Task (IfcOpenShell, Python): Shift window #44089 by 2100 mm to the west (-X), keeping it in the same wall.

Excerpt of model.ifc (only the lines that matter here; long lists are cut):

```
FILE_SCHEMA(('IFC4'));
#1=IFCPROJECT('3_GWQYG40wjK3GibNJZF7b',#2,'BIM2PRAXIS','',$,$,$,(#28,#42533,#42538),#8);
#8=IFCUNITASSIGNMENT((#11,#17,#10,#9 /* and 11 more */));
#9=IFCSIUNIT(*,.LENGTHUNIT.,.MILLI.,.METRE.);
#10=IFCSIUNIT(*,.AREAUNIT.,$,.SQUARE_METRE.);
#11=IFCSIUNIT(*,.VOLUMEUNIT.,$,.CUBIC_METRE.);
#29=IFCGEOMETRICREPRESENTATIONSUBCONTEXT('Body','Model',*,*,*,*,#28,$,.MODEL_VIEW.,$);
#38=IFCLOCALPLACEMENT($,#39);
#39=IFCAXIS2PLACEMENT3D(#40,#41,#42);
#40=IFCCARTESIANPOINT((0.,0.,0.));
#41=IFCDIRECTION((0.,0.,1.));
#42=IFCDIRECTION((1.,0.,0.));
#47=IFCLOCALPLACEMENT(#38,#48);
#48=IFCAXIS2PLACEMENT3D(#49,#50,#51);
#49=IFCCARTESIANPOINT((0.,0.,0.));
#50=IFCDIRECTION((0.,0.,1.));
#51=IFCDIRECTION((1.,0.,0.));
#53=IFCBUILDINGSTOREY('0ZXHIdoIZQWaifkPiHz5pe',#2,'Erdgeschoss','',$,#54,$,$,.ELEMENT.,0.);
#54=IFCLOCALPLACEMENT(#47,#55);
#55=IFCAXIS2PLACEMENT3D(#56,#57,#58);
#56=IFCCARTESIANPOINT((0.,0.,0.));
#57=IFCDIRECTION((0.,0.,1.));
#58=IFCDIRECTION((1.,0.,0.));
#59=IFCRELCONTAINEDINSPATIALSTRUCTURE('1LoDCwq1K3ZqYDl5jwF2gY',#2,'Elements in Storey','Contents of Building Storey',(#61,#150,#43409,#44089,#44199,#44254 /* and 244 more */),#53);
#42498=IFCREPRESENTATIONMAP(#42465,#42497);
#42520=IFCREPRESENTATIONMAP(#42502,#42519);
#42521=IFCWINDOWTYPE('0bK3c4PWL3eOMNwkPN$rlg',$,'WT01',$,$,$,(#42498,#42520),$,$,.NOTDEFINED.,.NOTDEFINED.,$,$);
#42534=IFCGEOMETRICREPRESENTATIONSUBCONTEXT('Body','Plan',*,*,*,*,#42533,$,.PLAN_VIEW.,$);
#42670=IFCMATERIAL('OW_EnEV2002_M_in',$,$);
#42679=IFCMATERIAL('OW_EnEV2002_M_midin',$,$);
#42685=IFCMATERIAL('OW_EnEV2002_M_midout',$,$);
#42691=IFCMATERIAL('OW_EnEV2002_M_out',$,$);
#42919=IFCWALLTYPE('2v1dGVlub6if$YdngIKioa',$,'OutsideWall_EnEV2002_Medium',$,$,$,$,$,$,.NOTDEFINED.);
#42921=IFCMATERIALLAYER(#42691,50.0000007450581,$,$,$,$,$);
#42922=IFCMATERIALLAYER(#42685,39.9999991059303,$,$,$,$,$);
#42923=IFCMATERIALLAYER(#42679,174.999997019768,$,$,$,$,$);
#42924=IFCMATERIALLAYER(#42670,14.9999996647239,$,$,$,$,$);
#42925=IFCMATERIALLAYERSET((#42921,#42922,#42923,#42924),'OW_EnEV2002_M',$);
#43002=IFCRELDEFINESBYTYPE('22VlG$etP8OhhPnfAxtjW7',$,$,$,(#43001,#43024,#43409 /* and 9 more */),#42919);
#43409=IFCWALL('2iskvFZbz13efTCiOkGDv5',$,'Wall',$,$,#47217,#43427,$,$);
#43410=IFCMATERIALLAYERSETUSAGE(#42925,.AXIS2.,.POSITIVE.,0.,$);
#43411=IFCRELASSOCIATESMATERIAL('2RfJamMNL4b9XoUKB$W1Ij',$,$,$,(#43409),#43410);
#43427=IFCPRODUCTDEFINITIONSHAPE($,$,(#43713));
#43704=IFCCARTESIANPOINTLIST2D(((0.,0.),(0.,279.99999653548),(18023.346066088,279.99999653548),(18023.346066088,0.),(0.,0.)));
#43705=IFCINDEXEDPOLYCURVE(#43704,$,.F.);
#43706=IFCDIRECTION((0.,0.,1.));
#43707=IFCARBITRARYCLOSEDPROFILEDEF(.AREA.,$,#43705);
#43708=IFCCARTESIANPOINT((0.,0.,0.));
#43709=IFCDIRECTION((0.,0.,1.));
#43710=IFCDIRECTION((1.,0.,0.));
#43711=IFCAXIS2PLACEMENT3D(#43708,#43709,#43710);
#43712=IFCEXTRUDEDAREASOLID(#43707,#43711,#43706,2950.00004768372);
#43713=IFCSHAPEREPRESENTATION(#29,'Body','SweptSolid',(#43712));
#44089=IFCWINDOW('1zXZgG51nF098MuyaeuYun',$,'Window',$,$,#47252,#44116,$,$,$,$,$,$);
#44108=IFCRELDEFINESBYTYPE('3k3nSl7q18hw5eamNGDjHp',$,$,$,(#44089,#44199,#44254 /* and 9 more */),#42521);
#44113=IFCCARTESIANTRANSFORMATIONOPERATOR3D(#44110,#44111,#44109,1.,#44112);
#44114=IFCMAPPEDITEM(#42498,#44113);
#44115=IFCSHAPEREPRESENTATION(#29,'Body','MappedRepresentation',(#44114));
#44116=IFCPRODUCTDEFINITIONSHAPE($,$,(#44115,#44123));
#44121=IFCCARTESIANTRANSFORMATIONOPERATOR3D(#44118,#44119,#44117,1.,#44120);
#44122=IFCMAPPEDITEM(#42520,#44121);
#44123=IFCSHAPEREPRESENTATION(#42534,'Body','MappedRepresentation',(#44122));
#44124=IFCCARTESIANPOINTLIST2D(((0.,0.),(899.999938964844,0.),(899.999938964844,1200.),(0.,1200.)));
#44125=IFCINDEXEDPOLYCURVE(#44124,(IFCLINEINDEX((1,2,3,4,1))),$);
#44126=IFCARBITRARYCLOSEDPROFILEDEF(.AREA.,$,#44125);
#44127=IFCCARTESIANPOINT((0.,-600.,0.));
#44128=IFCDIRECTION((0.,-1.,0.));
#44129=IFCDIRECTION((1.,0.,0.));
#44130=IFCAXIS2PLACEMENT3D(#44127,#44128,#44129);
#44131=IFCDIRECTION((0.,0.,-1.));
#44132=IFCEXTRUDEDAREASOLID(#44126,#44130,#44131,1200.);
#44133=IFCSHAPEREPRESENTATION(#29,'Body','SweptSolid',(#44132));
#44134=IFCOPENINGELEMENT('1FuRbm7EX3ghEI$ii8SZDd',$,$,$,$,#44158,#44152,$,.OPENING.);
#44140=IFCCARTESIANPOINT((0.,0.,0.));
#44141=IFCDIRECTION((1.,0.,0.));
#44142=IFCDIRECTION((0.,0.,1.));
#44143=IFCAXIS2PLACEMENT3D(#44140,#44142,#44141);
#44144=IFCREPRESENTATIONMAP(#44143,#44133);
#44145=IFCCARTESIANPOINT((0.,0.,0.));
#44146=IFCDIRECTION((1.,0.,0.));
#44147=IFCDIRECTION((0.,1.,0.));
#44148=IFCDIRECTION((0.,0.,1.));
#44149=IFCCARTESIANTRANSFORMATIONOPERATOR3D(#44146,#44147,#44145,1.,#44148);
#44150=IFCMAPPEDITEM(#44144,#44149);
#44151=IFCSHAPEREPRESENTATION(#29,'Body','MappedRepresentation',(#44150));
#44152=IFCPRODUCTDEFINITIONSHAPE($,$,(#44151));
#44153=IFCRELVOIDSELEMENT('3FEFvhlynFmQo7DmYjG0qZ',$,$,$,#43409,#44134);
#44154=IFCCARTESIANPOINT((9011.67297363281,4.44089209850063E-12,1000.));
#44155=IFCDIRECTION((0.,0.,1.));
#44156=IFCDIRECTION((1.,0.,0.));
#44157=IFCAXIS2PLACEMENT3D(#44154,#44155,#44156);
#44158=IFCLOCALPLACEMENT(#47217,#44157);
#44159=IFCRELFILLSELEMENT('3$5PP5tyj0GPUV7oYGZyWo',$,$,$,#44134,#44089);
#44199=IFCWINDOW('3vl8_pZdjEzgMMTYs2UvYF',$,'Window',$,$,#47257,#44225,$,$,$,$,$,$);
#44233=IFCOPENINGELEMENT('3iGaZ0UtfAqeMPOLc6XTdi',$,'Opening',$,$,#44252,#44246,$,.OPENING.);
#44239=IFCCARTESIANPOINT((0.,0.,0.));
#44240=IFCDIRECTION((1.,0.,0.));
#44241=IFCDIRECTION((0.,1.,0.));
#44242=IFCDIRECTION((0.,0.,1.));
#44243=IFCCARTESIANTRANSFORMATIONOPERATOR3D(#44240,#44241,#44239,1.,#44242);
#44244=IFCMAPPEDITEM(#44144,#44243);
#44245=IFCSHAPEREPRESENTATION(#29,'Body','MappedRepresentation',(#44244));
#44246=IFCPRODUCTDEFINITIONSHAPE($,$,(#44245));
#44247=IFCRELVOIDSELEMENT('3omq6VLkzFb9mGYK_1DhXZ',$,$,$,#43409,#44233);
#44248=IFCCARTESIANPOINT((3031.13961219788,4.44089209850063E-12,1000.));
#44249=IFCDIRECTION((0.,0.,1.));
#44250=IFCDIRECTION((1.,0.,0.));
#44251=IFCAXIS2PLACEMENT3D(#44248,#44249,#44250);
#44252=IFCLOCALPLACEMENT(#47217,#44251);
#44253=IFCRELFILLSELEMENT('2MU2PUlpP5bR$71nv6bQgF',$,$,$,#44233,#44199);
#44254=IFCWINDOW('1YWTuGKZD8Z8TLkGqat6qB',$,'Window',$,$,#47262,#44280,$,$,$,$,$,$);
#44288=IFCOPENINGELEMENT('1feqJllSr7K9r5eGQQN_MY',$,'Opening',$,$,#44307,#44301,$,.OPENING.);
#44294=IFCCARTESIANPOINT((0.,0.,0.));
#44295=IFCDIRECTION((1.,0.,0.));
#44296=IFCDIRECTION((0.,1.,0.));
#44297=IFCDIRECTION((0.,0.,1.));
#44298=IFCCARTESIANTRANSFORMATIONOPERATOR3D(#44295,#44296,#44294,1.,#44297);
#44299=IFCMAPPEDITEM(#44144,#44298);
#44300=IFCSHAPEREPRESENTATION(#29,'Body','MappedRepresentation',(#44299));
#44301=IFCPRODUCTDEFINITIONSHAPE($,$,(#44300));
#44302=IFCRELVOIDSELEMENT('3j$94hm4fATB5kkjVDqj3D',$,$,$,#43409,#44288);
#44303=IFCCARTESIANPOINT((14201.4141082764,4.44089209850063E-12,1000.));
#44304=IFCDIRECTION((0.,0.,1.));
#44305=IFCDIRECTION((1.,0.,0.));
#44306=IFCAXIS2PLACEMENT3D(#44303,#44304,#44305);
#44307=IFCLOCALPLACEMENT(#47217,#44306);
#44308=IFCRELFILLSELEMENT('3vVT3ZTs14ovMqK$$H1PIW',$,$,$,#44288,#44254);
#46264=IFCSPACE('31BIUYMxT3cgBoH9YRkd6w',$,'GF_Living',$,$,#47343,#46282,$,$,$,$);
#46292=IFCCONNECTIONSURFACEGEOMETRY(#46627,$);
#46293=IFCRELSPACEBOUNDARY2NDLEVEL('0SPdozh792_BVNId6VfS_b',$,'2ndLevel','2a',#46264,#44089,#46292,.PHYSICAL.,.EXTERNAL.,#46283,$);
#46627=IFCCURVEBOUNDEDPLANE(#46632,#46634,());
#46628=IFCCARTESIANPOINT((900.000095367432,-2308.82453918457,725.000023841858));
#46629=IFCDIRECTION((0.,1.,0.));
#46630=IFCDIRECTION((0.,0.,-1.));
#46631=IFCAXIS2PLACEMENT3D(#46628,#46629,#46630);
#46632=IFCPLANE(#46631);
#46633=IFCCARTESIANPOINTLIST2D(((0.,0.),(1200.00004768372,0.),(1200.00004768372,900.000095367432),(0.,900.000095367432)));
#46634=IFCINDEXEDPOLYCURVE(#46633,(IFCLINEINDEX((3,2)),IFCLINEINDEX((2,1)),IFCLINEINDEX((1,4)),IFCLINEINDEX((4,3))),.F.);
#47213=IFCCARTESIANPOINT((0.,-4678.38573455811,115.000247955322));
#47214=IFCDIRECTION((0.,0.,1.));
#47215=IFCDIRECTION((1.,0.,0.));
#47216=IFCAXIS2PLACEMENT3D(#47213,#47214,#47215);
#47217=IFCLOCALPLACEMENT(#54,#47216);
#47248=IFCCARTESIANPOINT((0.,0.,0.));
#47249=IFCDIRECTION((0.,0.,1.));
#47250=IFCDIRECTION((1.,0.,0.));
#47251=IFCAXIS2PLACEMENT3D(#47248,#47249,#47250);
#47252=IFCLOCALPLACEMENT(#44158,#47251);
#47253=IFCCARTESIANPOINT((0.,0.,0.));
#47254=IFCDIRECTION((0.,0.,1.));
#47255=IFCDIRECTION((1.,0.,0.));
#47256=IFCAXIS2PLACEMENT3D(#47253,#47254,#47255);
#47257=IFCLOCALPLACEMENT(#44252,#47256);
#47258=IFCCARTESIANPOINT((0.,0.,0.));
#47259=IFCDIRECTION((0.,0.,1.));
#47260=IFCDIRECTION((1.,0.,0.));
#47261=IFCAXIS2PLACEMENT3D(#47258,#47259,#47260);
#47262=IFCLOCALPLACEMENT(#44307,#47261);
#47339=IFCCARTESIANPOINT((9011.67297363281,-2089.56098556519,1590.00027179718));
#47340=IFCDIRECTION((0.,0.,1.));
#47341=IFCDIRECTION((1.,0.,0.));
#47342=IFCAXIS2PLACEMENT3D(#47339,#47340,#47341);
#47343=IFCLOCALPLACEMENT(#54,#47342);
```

```python
import numpy as np
import ifcopenshell
import ifcopenshell.api.geometry
import ifcopenshell.util.placement

model = ifcopenshell.open("model.ifc")

window = model.by_guid("1zXZgG51nF098MuyaeuYun")
opening = window.FillsVoids[0].RelatingOpeningElement
wall = opening.VoidsElements[0].RelatingBuildingElement

wall_matrix = ifcopenshell.util.placement.get_local_placement(wall.ObjectPlacement)
shift = wall_matrix[:3, 0] * -2100.0
before = ifcopenshell.util.placement.get_local_placement(window.ObjectPlacement)[:3, 3].copy()

# The window is placed relative to its opening, so it follows when the opening moves.
matrix = ifcopenshell.util.placement.get_local_placement(opening.ObjectPlacement)
matrix[:3, 3] += shift
ifcopenshell.api.geometry.edit_object_placement(
    model, product=opening, matrix=matrix, is_si=False, should_transform_children=True
)

# Space boundary surfaces are stored in each space's coordinates; move them too.
for rel in window.ProvidesBoundaries:
    if not rel.ConnectionGeometry:
        continue
    surface = rel.ConnectionGeometry.SurfaceOnRelatingElement.BasisSurface
    space_matrix = ifcopenshell.util.placement.get_local_placement(rel.RelatingSpace.ObjectPlacement)
    point = np.array(surface.Position.Location.Coordinates) + space_matrix[:3, :3].T @ shift
    surface.Position = model.createIfcAxis2Placement3D(
        model.createIfcCartesianPoint(point.tolist()), surface.Position.Axis, surface.Position.RefDirection
    )

after = ifcopenshell.util.placement.get_local_placement(window.ObjectPlacement)[:3, 3]
print("window moved by", (after - before).round(3) + 0.0)

model.write("model_rev.ifc")
```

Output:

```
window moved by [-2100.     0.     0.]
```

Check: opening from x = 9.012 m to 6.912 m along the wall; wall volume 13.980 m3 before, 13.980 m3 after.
